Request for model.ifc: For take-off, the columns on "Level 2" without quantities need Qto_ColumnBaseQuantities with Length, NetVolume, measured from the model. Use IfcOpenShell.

First a look at what the model holds.

```python
import ifcopenshell
import ifcopenshell.util.element
import ifcopenshell.util.unit

model = ifcopenshell.open("model.ifc")
print(model.schema)
for unit_type in ("LENGTHUNIT", "AREAUNIT", "VOLUMEUNIT"):
    print(unit_type, ifcopenshell.util.unit.calculate_unit_scale(model, unit_type))
storey = next(s for s in model.by_type("IfcBuildingStorey") if s.Name == "Level 2")
columns = [e for e in ifcopenshell.util.element.get_decomposition(storey) if e.is_a("IfcColumn")]
for e in sorted(columns, key=lambda e: e.id()):
    print(e.id(), e.is_a(), e.Name, list(ifcopenshell.util.element.get_psets(e, qtos_only=True)), sep=" | ")
```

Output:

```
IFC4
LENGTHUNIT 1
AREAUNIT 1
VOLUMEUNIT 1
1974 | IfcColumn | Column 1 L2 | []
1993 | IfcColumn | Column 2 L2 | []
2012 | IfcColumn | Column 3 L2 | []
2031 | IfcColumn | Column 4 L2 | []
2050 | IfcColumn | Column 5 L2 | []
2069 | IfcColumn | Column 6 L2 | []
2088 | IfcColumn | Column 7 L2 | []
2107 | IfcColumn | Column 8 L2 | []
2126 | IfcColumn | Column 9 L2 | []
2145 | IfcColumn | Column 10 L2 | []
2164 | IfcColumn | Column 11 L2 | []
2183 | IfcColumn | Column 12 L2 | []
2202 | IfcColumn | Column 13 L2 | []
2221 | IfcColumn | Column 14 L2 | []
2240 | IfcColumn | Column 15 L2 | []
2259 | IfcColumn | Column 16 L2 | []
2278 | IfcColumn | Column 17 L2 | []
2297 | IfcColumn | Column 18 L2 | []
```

```python
import ifcopenshell
import ifcopenshell.api.pset
import ifcopenshell.geom
import ifcopenshell.util.element
import ifcopenshell.util.shape
import ifcopenshell.util.unit

model = ifcopenshell.open("model.ifc")
unit_scale = ifcopenshell.util.unit.calculate_unit_scale(model)
volume_scale = ifcopenshell.util.unit.calculate_unit_scale(model, "VOLUMEUNIT")
settings = ifcopenshell.geom.settings()

storey = next(s for s in model.by_type("IfcBuildingStorey") if s.Name == "Level 2")
columns = [e for e in ifcopenshell.util.element.get_decomposition(storey) if e.is_a("IfcColumn")]

for e in sorted(columns, key=lambda e: e.id()):
    if ifcopenshell.util.element.get_psets(e, qtos_only=True, should_inherit=False):
        continue
    # Geometry comes back in metres, in the element's own axes.
    shape = ifcopenshell.geom.create_shape(settings, e)
    values = {
        "Length": ifcopenshell.util.shape.get_z(shape.geometry) / unit_scale,
        "NetVolume": ifcopenshell.util.shape.get_volume(shape.geometry) / volume_scale,
    }
    qto = ifcopenshell.api.pset.add_qto(model, product=e, name="Qto_ColumnBaseQuantities")
    ifcopenshell.api.pset.edit_qto(model, qto=qto, properties=values)
    print(e.id(), {k: round(v, 3) for k, v in values.items()})

model.write("model_updated.ifc")
```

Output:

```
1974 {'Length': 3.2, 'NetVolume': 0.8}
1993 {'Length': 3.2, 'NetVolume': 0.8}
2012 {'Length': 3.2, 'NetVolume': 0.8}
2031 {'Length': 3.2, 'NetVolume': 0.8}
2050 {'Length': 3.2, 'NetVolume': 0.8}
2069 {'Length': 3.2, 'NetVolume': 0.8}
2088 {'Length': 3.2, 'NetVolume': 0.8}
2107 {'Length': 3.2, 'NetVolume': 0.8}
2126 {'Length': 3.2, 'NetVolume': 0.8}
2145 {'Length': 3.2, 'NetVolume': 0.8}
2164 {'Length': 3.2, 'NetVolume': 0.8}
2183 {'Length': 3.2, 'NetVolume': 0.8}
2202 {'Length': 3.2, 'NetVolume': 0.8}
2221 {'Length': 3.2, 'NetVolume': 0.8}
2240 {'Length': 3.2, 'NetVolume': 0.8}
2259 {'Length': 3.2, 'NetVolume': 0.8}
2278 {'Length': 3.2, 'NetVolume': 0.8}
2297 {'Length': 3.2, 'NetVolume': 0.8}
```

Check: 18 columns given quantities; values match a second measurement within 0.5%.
